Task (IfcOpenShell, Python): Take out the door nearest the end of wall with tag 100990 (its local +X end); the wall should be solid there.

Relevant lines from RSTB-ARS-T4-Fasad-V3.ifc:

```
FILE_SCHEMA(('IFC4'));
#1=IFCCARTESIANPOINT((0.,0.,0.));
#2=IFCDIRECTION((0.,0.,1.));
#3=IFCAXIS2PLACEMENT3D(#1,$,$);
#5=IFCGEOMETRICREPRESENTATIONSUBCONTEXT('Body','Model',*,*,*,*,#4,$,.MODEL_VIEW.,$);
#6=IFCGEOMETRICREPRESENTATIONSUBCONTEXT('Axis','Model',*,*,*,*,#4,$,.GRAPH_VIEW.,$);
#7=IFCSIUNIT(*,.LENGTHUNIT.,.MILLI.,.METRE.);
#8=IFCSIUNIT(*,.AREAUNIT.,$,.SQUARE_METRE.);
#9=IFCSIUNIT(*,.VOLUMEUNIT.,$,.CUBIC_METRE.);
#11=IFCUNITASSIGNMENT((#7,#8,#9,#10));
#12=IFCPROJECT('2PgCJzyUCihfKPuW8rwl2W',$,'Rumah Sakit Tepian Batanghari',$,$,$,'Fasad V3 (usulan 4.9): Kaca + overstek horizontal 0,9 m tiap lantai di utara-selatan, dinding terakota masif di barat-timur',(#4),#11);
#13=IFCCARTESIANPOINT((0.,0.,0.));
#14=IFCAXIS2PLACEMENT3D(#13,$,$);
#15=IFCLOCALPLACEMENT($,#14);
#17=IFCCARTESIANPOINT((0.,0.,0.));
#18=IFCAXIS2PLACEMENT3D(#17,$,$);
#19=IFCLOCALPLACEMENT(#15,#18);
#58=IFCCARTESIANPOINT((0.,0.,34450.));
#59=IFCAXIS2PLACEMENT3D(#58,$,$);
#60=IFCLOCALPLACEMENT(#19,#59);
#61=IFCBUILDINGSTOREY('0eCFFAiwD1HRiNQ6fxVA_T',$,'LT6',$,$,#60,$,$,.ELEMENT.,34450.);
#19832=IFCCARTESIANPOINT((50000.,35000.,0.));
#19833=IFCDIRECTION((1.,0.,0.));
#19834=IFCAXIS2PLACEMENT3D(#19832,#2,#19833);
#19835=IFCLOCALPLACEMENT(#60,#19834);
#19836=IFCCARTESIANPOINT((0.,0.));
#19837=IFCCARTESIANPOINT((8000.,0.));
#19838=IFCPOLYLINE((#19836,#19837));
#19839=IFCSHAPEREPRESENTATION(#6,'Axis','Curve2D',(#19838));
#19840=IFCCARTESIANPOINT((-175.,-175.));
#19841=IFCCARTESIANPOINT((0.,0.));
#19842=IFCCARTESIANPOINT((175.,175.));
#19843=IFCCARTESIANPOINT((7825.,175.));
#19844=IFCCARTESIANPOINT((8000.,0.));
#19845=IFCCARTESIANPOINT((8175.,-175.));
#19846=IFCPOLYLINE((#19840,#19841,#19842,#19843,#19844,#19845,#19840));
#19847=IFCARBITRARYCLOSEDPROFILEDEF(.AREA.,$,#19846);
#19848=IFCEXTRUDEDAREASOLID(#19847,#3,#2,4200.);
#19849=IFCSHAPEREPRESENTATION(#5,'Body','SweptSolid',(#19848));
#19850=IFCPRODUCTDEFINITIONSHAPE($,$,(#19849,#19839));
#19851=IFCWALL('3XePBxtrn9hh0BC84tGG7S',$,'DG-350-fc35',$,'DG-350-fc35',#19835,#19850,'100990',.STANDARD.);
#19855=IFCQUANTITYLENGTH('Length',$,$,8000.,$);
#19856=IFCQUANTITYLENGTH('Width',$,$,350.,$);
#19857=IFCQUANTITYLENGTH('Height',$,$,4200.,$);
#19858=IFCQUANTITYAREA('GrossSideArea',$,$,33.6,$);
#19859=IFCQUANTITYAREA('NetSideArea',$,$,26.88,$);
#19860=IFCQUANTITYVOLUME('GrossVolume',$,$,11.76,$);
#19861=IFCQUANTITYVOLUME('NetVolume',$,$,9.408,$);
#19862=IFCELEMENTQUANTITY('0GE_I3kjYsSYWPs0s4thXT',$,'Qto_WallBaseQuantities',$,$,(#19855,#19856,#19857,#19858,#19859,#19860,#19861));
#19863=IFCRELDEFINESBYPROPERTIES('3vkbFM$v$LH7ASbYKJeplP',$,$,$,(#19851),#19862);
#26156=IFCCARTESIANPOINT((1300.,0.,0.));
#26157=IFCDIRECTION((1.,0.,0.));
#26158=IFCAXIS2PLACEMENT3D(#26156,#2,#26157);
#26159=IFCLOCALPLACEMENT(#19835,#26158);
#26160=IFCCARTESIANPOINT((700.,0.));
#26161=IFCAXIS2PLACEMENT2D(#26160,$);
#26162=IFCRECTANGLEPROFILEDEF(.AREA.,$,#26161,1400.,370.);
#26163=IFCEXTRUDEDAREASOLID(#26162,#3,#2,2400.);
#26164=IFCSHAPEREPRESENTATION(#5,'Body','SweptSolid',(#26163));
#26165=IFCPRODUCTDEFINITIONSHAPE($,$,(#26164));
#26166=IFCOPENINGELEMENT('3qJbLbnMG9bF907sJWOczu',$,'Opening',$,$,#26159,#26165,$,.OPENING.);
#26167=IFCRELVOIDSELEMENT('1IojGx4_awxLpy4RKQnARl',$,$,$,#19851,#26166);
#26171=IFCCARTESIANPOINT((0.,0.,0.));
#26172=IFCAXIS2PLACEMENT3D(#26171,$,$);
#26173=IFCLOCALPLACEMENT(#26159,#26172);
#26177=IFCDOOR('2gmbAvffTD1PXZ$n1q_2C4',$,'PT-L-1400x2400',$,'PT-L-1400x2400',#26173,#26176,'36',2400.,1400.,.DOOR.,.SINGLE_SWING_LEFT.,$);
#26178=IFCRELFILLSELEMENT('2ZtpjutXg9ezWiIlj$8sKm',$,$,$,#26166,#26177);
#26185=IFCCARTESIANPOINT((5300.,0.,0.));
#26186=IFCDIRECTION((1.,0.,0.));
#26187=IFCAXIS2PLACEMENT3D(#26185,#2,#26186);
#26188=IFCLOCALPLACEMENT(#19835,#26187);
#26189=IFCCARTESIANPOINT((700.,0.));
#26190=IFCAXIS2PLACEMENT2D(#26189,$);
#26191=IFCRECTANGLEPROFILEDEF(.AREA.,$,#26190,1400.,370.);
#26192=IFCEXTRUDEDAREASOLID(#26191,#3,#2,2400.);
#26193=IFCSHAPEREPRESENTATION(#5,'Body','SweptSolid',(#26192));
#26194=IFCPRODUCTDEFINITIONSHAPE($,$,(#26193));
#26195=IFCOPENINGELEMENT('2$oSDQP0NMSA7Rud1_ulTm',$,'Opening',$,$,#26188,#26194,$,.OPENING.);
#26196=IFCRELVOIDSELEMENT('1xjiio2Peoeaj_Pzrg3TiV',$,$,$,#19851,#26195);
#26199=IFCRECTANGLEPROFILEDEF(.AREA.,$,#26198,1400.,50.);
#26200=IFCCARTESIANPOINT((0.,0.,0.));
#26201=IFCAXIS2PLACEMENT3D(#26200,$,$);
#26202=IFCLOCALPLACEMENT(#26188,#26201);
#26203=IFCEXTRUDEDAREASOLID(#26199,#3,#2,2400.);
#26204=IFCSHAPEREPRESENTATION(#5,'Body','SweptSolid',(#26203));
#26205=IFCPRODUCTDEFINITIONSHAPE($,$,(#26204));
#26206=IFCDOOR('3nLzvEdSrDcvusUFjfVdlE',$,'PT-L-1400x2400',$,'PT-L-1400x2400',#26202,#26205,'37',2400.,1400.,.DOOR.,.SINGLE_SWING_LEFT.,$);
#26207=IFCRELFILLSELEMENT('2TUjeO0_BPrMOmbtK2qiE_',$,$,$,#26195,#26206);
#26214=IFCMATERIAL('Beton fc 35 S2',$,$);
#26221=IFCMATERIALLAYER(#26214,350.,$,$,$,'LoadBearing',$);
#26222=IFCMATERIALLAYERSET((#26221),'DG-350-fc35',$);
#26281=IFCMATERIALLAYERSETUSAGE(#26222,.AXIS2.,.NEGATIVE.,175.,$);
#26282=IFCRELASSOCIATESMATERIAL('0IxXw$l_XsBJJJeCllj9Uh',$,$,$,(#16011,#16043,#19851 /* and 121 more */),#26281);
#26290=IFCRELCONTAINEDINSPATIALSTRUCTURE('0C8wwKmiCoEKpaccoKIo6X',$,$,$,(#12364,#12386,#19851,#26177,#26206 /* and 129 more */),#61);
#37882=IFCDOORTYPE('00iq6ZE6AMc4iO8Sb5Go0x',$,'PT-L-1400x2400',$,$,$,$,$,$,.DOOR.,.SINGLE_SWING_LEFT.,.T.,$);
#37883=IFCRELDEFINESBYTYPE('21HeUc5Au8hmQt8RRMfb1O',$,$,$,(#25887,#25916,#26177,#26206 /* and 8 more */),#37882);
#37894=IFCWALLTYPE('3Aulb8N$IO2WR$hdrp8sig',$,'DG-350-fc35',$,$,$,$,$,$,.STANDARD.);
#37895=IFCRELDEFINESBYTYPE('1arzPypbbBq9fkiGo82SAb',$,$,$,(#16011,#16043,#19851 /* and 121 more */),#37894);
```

```python
import ifcopenshell
import ifcopenshell.api.feature
import ifcopenshell.api.pset
import ifcopenshell.api.root
import ifcopenshell.geom
import ifcopenshell.util.element
import ifcopenshell.util.shape
import ifcopenshell.util.unit

model = ifcopenshell.open("RSTB-ARS-T4-Fasad-V3.ifc")
area_scale = ifcopenshell.util.unit.calculate_unit_scale(model, "AREAUNIT")
volume_scale = ifcopenshell.util.unit.calculate_unit_scale(model, "VOLUMEUNIT")
settings = ifcopenshell.geom.settings()


def volume(element):
    """Net volume in cubic metres, openings subtracted."""
    shape = ifcopenshell.geom.create_shape(settings, element)
    return ifcopenshell.util.shape.get_volume(shape.geometry)


door = model.by_id(26206)
opening = door.FillsVoids[0].RelatingOpeningElement
wall = opening.VoidsElements[0].RelatingBuildingElement
before = volume(wall)

ifcopenshell.api.root.remove_product(model, product=door)
ifcopenshell.api.feature.remove_feature(model, feature=opening)

after = volume(wall)
thickness = 0.35  # wall thickness in metres

# Update the wall's stored quantities.
qto = model.by_id(ifcopenshell.util.element.get_pset(wall, "Qto_WallBaseQuantities", should_inherit=False)["id"])
ifcopenshell.api.pset.edit_qto(model, qto=qto, properties={
    "NetSideArea": after / thickness / area_scale,
    "NetVolume": after / volume_scale,
})

print(f"wall volume {before:.3f} -> {after:.3f} m3")

model.write("RSTB-ARS-T4-Fasad-V3_rev.ifc")
```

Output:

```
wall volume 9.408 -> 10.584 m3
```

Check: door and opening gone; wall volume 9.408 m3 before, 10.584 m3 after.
